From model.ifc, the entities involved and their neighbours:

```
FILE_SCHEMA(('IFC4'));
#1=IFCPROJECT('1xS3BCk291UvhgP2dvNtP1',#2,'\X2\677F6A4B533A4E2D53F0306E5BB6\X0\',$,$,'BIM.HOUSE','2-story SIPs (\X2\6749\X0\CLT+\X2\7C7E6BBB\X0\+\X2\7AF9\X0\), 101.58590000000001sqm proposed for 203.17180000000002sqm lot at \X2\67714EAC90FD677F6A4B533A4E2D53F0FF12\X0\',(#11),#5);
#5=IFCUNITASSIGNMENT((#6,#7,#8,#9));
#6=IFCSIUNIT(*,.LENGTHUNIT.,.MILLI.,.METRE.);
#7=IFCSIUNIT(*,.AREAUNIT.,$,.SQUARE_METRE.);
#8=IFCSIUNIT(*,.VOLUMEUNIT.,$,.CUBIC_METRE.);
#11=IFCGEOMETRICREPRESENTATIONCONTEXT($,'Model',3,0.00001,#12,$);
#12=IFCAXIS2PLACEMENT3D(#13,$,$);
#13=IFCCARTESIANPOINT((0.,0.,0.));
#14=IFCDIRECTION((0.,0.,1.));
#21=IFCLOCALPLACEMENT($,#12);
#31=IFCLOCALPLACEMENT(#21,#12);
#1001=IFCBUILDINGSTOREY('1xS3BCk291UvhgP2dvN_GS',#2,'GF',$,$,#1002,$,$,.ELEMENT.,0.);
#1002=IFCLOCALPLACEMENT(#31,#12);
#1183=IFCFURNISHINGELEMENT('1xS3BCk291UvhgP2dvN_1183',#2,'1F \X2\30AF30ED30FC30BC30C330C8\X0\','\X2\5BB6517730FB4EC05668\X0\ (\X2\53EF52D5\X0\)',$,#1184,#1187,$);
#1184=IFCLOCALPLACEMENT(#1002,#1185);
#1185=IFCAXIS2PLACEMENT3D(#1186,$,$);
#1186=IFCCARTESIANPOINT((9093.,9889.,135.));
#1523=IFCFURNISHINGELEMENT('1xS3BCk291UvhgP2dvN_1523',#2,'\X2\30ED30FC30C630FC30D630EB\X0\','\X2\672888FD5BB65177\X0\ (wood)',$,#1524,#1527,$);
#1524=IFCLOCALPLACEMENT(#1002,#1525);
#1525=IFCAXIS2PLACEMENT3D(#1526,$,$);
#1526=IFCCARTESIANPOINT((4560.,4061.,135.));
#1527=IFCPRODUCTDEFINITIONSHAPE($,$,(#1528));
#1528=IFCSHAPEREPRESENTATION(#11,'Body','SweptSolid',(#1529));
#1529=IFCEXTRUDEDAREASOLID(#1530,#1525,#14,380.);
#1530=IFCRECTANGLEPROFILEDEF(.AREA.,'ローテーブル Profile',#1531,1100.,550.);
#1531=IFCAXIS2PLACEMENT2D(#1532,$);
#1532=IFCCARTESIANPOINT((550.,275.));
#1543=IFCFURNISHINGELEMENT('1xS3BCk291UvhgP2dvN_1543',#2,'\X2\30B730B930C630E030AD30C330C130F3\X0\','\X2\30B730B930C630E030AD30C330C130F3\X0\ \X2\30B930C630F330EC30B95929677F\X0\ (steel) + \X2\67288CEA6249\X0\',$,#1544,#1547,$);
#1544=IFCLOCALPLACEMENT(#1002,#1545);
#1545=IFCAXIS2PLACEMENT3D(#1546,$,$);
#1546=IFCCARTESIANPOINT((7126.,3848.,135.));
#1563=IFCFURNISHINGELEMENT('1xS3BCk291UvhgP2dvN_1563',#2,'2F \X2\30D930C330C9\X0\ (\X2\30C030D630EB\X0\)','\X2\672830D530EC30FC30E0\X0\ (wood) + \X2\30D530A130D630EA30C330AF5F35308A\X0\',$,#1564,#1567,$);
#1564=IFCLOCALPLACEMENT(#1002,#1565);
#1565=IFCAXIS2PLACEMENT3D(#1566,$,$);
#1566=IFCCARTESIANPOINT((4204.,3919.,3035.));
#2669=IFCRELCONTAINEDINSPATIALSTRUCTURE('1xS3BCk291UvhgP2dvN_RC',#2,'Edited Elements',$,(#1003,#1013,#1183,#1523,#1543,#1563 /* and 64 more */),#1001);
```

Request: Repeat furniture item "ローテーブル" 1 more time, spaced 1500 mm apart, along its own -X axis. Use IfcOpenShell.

```python
import ifcopenshell
import ifcopenshell.api.geometry
import ifcopenshell.api.root
import ifcopenshell.util.element
import ifcopenshell.util.placement

model = ifcopenshell.open("model.ifc")


def reuse_history(source, copy):
    """copy_class also copies each property set's owner history, people and application; keep the originals."""
    for rel in copy.IsDefinedBy:
        if rel.is_a("IfcRelDefinesByProperties") and (history := rel.RelatingPropertyDefinition.OwnerHistory):
            rel.RelatingPropertyDefinition.OwnerHistory = source.OwnerHistory
            ifcopenshell.util.element.remove_deep2(model, history)


source = model.by_guid("1xS3BCk291UvhgP2dvN_1523")
base = ifcopenshell.util.placement.get_local_placement(source.ObjectPlacement)
step = -base[:3, 0] * 1500.0

for i in range(1, 2):
    copy = ifcopenshell.api.root.copy_class(model, product=source)
    copy.Representation = ifcopenshell.util.element.copy_deep(
        model, source.Representation, exclude=["IfcGeometricRepresentationContext", "IfcRepresentationMap"]
    )
    reuse_history(source, copy)
    matrix = base.copy()
    matrix[:3, 3] += i * step
    print("added at", matrix[:3, 3].round(3) + 0.0)
    ifcopenshell.api.geometry.edit_object_placement(model, product=copy, matrix=matrix, is_si=False)

model.write("model-out.ifc")
```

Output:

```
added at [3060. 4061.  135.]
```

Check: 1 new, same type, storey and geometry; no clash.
